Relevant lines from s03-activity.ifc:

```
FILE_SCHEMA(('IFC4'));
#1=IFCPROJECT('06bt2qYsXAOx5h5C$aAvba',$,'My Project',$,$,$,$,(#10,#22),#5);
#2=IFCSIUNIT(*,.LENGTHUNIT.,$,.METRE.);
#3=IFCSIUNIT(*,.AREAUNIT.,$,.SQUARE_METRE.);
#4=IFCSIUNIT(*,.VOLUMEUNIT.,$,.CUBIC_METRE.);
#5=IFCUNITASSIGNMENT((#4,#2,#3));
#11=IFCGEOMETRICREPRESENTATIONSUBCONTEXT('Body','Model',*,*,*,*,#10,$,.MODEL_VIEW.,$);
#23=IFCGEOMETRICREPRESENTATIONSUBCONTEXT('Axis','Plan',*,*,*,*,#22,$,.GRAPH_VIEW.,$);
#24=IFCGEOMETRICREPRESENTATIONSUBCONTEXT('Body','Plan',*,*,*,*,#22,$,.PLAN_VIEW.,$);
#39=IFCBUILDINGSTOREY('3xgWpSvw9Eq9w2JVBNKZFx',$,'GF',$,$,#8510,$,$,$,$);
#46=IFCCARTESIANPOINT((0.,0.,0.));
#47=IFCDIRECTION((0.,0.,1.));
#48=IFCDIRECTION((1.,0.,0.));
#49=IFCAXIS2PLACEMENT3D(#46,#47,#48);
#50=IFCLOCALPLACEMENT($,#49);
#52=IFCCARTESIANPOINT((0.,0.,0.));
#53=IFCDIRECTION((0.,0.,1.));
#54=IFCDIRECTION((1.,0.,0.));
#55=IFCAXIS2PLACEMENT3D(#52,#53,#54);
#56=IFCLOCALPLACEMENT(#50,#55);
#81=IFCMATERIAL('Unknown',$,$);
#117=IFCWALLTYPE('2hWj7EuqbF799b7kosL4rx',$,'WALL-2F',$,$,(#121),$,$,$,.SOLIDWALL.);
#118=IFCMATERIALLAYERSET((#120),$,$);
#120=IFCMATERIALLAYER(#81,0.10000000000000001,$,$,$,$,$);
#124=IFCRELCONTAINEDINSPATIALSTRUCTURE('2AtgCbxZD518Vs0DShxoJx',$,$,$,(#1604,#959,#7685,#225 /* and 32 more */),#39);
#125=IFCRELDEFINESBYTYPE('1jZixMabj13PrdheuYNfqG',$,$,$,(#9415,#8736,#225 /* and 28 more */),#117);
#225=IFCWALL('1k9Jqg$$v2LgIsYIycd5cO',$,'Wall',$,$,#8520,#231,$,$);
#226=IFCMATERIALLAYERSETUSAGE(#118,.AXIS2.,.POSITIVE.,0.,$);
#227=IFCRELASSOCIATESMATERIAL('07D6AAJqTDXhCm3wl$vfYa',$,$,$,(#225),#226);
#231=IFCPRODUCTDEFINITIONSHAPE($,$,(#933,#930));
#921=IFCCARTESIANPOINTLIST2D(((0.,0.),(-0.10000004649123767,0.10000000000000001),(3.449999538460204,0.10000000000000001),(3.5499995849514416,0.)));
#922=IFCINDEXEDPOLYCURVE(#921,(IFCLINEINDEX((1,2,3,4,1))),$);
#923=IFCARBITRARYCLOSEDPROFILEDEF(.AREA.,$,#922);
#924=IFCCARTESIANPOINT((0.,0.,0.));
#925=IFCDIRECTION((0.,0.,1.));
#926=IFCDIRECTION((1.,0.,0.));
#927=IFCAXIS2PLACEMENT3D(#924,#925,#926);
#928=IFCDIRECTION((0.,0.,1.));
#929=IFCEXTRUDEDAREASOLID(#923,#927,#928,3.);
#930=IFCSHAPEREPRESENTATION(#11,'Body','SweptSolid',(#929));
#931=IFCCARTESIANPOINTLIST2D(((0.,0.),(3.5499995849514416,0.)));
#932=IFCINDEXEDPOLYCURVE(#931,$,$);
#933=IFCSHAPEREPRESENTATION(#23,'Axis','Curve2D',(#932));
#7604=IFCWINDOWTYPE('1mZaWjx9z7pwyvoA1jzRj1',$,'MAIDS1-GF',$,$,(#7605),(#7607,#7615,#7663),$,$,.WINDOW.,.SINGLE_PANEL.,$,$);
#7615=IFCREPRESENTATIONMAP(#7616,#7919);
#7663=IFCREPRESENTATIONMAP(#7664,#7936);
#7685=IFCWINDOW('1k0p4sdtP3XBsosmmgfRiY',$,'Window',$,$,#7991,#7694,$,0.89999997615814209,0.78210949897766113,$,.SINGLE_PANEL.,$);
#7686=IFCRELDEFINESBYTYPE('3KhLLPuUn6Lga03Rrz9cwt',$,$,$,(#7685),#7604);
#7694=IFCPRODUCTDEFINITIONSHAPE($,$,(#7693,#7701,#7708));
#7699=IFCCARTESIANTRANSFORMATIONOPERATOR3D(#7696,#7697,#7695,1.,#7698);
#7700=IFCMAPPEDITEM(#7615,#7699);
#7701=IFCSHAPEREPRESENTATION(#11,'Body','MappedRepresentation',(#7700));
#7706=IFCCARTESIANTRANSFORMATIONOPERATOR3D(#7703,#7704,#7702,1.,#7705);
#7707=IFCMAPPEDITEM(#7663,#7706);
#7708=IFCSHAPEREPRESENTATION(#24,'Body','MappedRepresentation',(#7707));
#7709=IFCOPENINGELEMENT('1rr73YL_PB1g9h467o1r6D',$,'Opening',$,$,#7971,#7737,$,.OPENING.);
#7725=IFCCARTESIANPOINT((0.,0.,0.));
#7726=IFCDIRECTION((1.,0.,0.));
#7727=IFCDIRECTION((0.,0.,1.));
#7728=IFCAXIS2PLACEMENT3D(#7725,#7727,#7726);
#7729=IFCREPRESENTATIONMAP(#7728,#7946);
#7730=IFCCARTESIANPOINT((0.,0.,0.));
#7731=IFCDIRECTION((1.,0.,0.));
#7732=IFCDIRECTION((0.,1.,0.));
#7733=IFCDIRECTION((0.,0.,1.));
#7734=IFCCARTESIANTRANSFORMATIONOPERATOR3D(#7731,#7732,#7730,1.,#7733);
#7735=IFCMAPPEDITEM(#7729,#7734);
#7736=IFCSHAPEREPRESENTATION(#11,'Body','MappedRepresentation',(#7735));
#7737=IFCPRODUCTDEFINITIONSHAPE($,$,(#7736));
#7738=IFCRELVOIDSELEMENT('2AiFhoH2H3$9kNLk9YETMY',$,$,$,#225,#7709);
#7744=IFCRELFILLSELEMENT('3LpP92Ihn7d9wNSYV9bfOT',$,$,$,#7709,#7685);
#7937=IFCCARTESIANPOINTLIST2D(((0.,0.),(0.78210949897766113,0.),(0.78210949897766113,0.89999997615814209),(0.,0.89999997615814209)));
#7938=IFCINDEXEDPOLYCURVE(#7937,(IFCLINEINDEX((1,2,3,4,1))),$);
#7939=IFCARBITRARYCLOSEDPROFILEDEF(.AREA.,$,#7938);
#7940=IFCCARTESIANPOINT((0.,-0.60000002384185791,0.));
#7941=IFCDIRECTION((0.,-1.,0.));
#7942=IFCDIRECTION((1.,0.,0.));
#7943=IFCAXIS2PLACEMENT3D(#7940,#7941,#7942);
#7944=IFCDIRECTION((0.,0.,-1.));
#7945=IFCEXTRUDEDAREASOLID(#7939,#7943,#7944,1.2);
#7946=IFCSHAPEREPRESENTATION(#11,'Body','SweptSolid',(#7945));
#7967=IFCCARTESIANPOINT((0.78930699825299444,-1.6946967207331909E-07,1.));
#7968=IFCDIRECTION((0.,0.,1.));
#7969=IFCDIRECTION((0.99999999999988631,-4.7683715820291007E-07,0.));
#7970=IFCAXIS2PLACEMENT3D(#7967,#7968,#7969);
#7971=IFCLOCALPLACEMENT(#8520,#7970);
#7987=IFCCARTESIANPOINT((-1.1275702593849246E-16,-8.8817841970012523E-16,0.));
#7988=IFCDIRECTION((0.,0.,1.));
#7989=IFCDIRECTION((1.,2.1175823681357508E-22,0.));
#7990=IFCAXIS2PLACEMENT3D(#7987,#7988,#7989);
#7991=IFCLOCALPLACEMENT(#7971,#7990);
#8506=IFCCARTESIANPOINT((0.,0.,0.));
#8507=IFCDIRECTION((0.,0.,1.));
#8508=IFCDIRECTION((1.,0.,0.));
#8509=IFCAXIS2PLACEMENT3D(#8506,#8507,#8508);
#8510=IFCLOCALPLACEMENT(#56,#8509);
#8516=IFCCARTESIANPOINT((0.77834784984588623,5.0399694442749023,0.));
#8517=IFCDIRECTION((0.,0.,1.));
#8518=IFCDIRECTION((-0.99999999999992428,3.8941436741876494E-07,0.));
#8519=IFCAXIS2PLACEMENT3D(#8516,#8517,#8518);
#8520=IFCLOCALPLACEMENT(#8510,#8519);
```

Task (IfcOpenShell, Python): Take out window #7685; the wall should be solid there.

```python
import ifcopenshell
import ifcopenshell.api.feature
import ifcopenshell.api.root
import ifcopenshell.geom
import ifcopenshell.util.shape

model = ifcopenshell.open("s03-activity.ifc")
settings = ifcopenshell.geom.settings()


def volume(element):
    """Net volume in cubic metres, openings subtracted."""
    shape = ifcopenshell.geom.create_shape(settings, element)
    return ifcopenshell.util.shape.get_volume(shape.geometry)


window = model.by_id(7685)
opening = window.FillsVoids[0].RelatingOpeningElement
wall = opening.VoidsElements[0].RelatingBuildingElement
before = volume(wall)

ifcopenshell.api.root.remove_product(model, product=window)
ifcopenshell.api.feature.remove_feature(model, feature=opening)

after = volume(wall)

print(f"wall volume {before:.3f} -> {after:.3f} m3")

model.write("s03-activity_rev.ifc")
```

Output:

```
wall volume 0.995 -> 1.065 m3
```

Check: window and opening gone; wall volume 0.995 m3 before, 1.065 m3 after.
